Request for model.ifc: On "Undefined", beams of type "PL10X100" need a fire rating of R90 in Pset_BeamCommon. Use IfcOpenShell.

First a look at what the model holds.

```python
import ifcopenshell
import ifcopenshell.util.element

model = ifcopenshell.open("model.ifc")
print(model.schema)
storey = next(s for s in model.by_type("IfcBuildingStorey") if s.Name == "Undefined")
beams = [e for e in ifcopenshell.util.element.get_decomposition(storey) if e.is_a("IfcBeam")]
seen = {}
for e in beams:
    element_type = ifcopenshell.util.element.get_type(e)
    key = (element_type.Name if element_type != e and element_type else None, ifcopenshell.util.element.get_pset(e, "Pset_BeamCommon", "FireRating"))
    seen[key] = seen.get(key, 0) + 1
for (name, value), count in sorted(seen.items(), key=str):
    print(count, "x", name, "|", value)
```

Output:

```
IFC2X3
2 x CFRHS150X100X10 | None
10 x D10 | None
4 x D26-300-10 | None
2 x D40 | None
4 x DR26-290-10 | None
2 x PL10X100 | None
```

```python
import ifcopenshell
import ifcopenshell.api.pset
import ifcopenshell.util.element

model = ifcopenshell.open("model.ifc")

storey = next(s for s in model.by_type("IfcBuildingStorey") if s.Name == "Undefined")
beams = [e for e in ifcopenshell.util.element.get_decomposition(storey) if e.is_a("IfcBeam")]

count = 0
for e in beams:
    element_type = ifcopenshell.util.element.get_type(e)
    if element_type in (None, e) or element_type.Name != "PL10X100":
        continue
    found = ifcopenshell.util.element.get_pset(e, "Pset_BeamCommon", should_inherit=False)
    if found:
        pset = model.by_id(found["id"])
        if len(ifcopenshell.util.element.get_elements_by_pset(pset)) > 1:
            pset = ifcopenshell.api.pset.unshare_pset(model, products=[e], pset=pset)[0]
    else:
        pset = ifcopenshell.api.pset.add_pset(model, product=e, name="Pset_BeamCommon")
    ifcopenshell.api.pset.edit_pset(model, pset=pset, properties={"FireRating": "R90"})
    count += 1

print(count, "beams updated")

model.write("model-out.ifc")
```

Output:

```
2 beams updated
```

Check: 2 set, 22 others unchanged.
